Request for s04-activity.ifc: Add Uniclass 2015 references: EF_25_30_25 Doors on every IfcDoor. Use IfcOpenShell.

First a look at what the model holds.

```python
import ifcopenshell

model = ifcopenshell.open("s04-activity.ifc")
print(model.schema)
print("classifications:", [c.Name for c in model.by_type("IfcClassification")])
for ifc_class in ("IfcDoor", "IfcRoof", "IfcStair", "IfcWall", "IfcWindow"):
    print(ifc_class, len(model.by_type(ifc_class)))
```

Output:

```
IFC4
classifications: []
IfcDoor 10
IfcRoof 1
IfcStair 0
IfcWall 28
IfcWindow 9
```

```python
import ifcopenshell
import ifcopenshell.api.classification

model = ifcopenshell.open("s04-activity.ifc")

system = ifcopenshell.api.classification.add_classification(model, classification="Uniclass 2015")

codes = {
    "IfcDoor": ("EF_25_30_25", "Doors"),
}
for ifc_class, (code, name) in codes.items():
    products = model.by_type(ifc_class)
    ifcopenshell.api.classification.add_reference(
        model, products=products, classification=system, identification=code, name=name
    )
    print(code, len(products))

model.write("s04-activity_updated.ifc")
```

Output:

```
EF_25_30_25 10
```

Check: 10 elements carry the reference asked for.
